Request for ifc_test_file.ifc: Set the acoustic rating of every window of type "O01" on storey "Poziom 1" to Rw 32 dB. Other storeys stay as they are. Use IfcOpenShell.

First a look at what the model holds.

```python
import ifcopenshell
import ifcopenshell.util.element

model = ifcopenshell.open("ifc_test_file.ifc")
print(model.schema)
storey = next(s for s in model.by_type("IfcBuildingStorey") if s.Name == "Poziom 1")
windows = [e for e in ifcopenshell.util.element.get_decomposition(storey) if e.is_a("IfcWindow")]
seen = {}
for e in windows:
    element_type = ifcopenshell.util.element.get_type(e)
    key = (element_type.Name if element_type != e and element_type else None, ifcopenshell.util.element.get_pset(e, "Pset_WindowCommon", "AcousticRating"))
    seen[key] = seen.get(key, 0) + 1
for (name, value), count in sorted(seen.items(), key=str):
    print(count, "x", name, "|", value)
```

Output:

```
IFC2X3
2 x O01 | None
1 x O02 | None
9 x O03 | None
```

```python
import ifcopenshell
import ifcopenshell.api.pset
import ifcopenshell.util.element

model = ifcopenshell.open("ifc_test_file.ifc")

storey = next(s for s in model.by_type("IfcBuildingStorey") if s.Name == "Poziom 1")
windows = [e for e in ifcopenshell.util.element.get_decomposition(storey) if e.is_a("IfcWindow")]

count = 0
for e in windows:
    element_type = ifcopenshell.util.element.get_type(e)
    if element_type in (None, e) or element_type.Name != "O01":
        continue
    # add_pset returns the element's existing set when there is one.
    pset = ifcopenshell.api.pset.add_pset(model, product=e, name="Pset_WindowCommon")
    ifcopenshell.api.pset.edit_pset(model, pset=pset, properties={"AcousticRating": "Rw 32 dB"})
    count += 1

print(count, "windows updated")

model.write("ifc_test_file_updated.ifc")
```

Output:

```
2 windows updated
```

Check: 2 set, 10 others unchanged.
